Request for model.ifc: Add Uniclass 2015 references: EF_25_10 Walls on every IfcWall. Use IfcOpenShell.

First a look at what the model holds.

```python
import ifcopenshell

model = ifcopenshell.open("model.ifc")
print(model.schema)
print("classifications:", [c.Name for c in model.by_type("IfcClassification")])
for ifc_class in ("IfcDoor", "IfcRoof", "IfcStair", "IfcWall", "IfcWindow"):
    print(ifc_class, len(model.by_type(ifc_class)))
```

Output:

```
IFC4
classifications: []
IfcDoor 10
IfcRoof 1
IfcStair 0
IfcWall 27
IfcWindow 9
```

```python
import ifcopenshell
import ifcopenshell.api.classification

model = ifcopenshell.open("model.ifc")

system = ifcopenshell.api.classification.add_classification(model, classification="Uniclass 2015")

codes = {
    "IfcWall": ("EF_25_10", "Walls"),
}
for ifc_class, (code, name) in codes.items():
    products = model.by_type(ifc_class)
    ifcopenshell.api.classification.add_reference(
        model, products=products, classification=system, identification=code, name=name
    )
    print(code, len(products))

model.write("model_v2.ifc")
```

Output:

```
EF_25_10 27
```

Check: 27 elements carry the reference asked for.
